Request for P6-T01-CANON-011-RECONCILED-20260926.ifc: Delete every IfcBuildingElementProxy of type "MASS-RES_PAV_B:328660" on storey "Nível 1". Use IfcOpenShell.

First a look at what the model holds.

```python
import ifcopenshell
import ifcopenshell.util.element

model = ifcopenshell.open("P6-T01-CANON-011-RECONCILED-20260926.ifc")
print(model.schema)
storey = next(s for s in model.by_type("IfcBuildingStorey") if s.Name == "Nível 1")
proxies = [e for e in ifcopenshell.util.element.get_decomposition(storey) if e.is_a("IfcBuildingElementProxy")]
seen = {}
for e in proxies:
    element_type = ifcopenshell.util.element.get_type(e)
    name = element_type.Name if element_type not in (None, e) else None
    seen[name] = seen.get(name, 0) + 1
for name, count in sorted(seen.items(), key=str):
    print(count, "x", name)
```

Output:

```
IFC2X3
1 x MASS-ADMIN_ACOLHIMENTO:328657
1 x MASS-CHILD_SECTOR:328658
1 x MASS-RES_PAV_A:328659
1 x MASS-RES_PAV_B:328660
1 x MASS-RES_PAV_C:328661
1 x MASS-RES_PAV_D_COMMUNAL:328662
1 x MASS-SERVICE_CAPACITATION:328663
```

```python
import ifcopenshell
import ifcopenshell.api.root
import ifcopenshell.util.element

model = ifcopenshell.open("P6-T01-CANON-011-RECONCILED-20260926.ifc")

storey = next(s for s in model.by_type("IfcBuildingStorey") if s.Name == "Nível 1")
proxies = [e for e in ifcopenshell.util.element.get_decomposition(storey) if e.is_a("IfcBuildingElementProxy")]
targets = [e for e in proxies if (t := ifcopenshell.util.element.get_type(e)) not in (None, e) and t.Name == "MASS-RES_PAV_B:328660"]

for e in targets:
    ifcopenshell.api.root.remove_product(model, product=e)
print(len(targets), "removed")

model.write("P6-T01-CANON-011-RECONCILED-20260926_rev.ifc")
```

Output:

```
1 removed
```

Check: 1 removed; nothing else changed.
